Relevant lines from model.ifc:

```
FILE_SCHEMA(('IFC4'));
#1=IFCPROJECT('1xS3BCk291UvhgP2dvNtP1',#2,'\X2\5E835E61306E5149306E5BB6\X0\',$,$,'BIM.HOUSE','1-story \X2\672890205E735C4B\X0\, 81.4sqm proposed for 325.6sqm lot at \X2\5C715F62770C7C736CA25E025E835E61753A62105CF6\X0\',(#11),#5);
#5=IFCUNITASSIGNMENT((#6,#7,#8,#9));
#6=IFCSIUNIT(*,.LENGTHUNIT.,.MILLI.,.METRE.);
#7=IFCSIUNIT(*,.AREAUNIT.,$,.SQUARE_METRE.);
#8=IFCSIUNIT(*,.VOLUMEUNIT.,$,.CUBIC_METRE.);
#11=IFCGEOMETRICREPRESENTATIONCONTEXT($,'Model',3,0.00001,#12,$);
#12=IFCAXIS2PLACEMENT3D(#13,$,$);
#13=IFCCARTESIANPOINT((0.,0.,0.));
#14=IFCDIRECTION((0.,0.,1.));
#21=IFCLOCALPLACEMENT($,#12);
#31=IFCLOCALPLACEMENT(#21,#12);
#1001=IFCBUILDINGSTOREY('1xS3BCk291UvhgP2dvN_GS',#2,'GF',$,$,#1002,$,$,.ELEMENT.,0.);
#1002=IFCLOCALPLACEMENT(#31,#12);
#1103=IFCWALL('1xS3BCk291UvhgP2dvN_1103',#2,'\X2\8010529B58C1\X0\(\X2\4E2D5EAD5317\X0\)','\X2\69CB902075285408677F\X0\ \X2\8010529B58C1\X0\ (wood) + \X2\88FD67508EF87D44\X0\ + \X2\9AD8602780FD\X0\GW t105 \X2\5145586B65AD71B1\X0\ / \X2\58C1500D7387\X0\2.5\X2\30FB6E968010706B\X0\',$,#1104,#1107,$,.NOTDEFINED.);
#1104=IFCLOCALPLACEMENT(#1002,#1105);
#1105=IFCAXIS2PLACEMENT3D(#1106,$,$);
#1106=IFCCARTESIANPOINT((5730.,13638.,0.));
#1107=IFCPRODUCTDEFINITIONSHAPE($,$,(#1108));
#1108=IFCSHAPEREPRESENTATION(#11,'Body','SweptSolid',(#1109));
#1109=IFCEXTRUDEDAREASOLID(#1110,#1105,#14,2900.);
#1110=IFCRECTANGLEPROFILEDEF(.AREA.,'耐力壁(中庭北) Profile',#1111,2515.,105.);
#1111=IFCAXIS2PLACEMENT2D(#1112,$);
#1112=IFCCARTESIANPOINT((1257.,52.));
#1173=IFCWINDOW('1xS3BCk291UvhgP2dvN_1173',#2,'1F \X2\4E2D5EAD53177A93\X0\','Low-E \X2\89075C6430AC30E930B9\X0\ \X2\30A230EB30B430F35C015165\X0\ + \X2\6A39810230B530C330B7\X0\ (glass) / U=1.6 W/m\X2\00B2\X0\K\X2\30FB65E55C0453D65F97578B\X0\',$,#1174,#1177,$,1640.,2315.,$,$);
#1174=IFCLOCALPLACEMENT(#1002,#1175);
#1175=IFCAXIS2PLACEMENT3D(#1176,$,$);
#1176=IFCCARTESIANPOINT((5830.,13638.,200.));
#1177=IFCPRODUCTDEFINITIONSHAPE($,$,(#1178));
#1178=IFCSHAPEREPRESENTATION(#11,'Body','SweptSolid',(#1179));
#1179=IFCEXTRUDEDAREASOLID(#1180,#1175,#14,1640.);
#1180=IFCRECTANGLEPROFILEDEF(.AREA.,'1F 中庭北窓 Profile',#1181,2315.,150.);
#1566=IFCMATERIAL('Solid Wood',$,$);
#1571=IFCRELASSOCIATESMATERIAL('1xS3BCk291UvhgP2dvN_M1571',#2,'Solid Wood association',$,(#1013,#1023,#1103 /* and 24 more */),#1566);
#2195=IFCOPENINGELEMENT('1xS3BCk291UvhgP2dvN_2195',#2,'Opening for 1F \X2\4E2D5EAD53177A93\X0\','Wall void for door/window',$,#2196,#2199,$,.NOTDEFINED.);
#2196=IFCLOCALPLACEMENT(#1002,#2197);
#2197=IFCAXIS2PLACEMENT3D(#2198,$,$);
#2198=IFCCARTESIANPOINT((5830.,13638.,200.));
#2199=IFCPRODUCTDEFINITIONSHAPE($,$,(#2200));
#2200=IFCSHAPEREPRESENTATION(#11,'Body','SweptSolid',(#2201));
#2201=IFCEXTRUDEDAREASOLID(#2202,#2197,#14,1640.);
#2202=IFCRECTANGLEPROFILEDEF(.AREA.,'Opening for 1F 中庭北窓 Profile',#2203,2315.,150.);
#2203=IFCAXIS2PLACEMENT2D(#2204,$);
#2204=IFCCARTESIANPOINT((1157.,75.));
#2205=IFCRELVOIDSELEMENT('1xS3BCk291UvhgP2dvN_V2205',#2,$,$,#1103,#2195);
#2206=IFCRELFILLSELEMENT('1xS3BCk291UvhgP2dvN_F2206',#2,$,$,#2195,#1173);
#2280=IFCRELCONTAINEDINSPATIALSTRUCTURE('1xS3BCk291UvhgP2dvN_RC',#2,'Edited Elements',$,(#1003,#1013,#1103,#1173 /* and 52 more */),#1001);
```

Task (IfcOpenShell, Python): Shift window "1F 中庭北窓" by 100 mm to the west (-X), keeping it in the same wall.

```python
import ifcopenshell
import ifcopenshell.api.geometry
import ifcopenshell.util.placement

model = ifcopenshell.open("model.ifc")

window = model.by_id(1173)
opening = window.FillsVoids[0].RelatingOpeningElement
wall = opening.VoidsElements[0].RelatingBuildingElement

wall_matrix = ifcopenshell.util.placement.get_local_placement(wall.ObjectPlacement)
shift = wall_matrix[:3, 0] * -100.0
before = ifcopenshell.util.placement.get_local_placement(window.ObjectPlacement)[:3, 3].copy()

# The window is not placed relative to its opening, so move both.
for product in (opening, window):
    matrix = ifcopenshell.util.placement.get_local_placement(product.ObjectPlacement)
    matrix[:3, 3] += shift
    ifcopenshell.api.geometry.edit_object_placement(model, product=product, matrix=matrix, is_si=False)

after = ifcopenshell.util.placement.get_local_placement(window.ObjectPlacement)[:3, 3]
print("window moved by", (after - before).round(3) + 0.0)

model.write("model_v2.ifc")
```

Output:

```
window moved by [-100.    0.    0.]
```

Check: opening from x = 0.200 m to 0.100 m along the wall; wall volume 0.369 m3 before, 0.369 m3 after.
